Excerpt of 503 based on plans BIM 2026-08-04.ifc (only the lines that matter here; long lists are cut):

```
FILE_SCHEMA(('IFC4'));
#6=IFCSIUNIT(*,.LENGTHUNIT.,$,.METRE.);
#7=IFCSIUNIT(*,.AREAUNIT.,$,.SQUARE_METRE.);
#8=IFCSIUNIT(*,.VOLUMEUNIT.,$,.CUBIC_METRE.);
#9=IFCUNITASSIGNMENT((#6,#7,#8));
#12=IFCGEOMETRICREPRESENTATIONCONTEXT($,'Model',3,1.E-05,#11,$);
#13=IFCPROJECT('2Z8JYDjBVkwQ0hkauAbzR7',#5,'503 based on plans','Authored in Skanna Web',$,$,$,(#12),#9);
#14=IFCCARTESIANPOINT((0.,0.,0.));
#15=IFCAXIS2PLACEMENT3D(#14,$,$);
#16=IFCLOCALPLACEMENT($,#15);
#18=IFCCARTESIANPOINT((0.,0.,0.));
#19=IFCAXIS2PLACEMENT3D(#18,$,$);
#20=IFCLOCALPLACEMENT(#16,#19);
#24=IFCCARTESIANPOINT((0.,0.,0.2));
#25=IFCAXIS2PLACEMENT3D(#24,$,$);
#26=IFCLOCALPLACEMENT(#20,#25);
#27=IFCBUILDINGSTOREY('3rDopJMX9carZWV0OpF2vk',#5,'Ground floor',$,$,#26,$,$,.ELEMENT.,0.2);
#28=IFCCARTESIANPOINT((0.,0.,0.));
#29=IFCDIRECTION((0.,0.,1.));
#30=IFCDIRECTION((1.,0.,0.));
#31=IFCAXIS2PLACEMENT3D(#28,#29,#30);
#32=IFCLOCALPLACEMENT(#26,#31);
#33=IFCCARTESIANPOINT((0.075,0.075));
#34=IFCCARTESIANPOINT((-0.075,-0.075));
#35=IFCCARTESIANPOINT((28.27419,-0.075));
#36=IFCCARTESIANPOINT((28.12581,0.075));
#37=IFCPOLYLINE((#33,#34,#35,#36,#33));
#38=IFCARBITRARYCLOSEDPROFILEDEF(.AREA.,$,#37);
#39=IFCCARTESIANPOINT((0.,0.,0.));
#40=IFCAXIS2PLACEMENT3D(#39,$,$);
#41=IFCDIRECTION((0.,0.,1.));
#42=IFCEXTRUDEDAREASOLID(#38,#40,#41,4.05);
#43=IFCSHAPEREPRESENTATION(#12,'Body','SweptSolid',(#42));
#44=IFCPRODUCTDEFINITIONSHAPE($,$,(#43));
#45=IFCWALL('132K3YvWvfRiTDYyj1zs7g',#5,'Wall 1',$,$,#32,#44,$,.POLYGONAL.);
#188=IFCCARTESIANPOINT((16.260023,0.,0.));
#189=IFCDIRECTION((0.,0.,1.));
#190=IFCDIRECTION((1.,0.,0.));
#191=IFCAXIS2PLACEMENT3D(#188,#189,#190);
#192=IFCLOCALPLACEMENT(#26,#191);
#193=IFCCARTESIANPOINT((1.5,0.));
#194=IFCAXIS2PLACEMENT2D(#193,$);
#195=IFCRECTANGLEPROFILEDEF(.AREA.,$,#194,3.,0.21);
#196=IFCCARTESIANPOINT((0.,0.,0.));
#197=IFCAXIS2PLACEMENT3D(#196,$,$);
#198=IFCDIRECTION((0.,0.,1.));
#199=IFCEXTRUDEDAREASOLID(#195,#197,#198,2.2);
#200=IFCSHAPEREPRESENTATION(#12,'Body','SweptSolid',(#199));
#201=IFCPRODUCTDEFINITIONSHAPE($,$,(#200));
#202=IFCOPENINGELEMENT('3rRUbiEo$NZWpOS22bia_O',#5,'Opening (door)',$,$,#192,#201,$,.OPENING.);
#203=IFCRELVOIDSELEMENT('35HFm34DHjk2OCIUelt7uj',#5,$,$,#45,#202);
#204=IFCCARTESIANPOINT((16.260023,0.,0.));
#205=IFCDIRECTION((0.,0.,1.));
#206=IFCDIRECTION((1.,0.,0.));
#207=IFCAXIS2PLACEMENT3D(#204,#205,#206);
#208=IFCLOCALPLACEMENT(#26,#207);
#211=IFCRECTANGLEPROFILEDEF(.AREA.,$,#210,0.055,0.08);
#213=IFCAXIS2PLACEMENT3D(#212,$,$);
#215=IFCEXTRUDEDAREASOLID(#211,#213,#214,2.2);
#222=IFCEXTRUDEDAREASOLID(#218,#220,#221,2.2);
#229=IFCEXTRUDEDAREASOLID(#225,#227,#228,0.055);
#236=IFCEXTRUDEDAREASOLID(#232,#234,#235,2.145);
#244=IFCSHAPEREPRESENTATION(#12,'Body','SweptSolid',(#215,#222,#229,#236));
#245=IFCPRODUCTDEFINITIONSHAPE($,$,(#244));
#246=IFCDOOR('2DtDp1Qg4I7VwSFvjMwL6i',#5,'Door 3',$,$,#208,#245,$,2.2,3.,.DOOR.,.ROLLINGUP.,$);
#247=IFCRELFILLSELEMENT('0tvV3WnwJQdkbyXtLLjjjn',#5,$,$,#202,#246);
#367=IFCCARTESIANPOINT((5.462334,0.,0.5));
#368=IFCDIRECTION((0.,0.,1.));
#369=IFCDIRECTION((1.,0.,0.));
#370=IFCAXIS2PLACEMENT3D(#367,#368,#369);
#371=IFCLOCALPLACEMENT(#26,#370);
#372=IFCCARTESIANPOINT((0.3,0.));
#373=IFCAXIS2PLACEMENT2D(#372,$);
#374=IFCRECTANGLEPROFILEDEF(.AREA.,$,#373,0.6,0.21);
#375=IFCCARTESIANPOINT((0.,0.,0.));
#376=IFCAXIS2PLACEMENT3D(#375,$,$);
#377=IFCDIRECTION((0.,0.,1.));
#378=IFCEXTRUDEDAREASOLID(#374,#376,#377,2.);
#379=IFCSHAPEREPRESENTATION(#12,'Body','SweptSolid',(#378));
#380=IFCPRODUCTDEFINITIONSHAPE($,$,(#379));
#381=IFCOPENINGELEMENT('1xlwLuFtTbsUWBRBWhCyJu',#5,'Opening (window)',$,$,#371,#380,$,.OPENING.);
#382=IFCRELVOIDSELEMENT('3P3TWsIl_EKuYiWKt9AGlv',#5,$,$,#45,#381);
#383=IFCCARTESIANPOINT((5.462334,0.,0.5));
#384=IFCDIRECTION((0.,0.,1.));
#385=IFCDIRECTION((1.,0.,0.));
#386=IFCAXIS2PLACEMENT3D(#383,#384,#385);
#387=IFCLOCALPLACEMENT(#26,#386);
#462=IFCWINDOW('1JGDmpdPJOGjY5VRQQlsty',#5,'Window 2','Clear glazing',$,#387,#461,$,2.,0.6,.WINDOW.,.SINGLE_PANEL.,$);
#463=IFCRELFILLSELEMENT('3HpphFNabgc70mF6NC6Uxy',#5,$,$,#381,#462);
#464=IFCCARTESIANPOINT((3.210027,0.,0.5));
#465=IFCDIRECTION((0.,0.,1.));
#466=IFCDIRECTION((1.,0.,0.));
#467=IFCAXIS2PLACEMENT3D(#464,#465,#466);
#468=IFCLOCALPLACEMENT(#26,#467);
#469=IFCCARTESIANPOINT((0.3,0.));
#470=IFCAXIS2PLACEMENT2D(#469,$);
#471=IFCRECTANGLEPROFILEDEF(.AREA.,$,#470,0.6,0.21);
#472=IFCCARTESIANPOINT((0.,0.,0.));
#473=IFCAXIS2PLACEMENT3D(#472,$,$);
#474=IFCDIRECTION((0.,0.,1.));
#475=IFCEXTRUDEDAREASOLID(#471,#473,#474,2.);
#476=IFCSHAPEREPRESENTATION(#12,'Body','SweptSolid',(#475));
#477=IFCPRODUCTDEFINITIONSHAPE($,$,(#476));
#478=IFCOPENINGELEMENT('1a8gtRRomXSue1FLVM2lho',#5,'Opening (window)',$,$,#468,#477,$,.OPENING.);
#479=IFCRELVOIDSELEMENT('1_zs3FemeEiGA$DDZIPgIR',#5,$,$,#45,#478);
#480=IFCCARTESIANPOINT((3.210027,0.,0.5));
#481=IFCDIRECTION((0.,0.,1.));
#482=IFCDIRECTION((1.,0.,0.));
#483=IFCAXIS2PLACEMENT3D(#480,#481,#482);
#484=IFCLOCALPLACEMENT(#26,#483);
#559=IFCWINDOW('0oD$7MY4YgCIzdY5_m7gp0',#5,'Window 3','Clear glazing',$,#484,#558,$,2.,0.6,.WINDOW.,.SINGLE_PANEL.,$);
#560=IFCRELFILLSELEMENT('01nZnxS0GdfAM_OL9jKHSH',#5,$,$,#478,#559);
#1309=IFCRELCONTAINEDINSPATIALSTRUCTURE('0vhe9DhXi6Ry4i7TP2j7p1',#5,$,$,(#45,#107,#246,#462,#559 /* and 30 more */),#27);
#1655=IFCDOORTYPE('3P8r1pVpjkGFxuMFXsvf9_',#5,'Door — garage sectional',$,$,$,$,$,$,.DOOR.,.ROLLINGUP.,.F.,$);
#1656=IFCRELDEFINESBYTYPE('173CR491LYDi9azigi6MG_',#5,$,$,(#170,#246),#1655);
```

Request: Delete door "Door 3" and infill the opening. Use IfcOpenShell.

```python
import ifcopenshell
import ifcopenshell.api.feature
import ifcopenshell.api.root
import ifcopenshell.geom
import ifcopenshell.util.shape

model = ifcopenshell.open("503 based on plans BIM 2026-08-04.ifc")
settings = ifcopenshell.geom.settings()


def volume(element):
    """Net volume in cubic metres, openings subtracted."""
    shape = ifcopenshell.geom.create_shape(settings, element)
    return ifcopenshell.util.shape.get_volume(shape.geometry)


door = model.by_id(246)
opening = door.FillsVoids[0].RelatingOpeningElement
wall = opening.VoidsElements[0].RelatingBuildingElement
before = volume(wall)

ifcopenshell.api.root.remove_product(model, product=door)
ifcopenshell.api.feature.remove_feature(model, feature=opening)

after = volume(wall)

print(f"wall volume {before:.3f} -> {after:.3f} m3")

model.write("503 based on plans BIM 2026-08-04-out.ifc")
```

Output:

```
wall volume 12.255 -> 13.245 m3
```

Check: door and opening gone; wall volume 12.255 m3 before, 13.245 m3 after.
